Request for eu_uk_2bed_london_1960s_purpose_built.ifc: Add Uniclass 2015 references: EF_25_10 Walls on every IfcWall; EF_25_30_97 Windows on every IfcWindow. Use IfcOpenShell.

First a look at what the model holds.

```python
import ifcopenshell

model = ifcopenshell.open("eu_uk_2bed_london_1960s_purpose_built.ifc")
print(model.schema)
print("classifications:", [c.Name for c in model.by_type("IfcClassification")])
for ifc_class in ("IfcDoor", "IfcRoof", "IfcStair", "IfcWall", "IfcWindow"):
    print(ifc_class, len(model.by_type(ifc_class)))
```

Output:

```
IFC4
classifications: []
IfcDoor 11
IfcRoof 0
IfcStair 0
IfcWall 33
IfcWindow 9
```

```python
import ifcopenshell
import ifcopenshell.api.classification

model = ifcopenshell.open("eu_uk_2bed_london_1960s_purpose_built.ifc")

system = ifcopenshell.api.classification.add_classification(model, classification="Uniclass 2015")

codes = {
    "IfcWall": ("EF_25_10", "Walls"),
    "IfcWindow": ("EF_25_30_97", "Windows"),
}
for ifc_class, (code, name) in codes.items():
    products = model.by_type(ifc_class)
    ifcopenshell.api.classification.add_reference(
        model, products=products, classification=system, identification=code, name=name
    )
    print(code, len(products))

model.write("eu_uk_2bed_london_1960s_purpose_built_edited.ifc")
```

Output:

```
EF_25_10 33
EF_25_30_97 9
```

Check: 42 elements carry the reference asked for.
